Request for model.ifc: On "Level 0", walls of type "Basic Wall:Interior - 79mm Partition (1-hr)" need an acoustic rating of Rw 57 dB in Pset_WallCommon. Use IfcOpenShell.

First a look at what the model holds.

```python
import ifcopenshell
import ifcopenshell.util.element

model = ifcopenshell.open("model.ifc")
print(model.schema)
storey = next(s for s in model.by_type("IfcBuildingStorey") if s.Name == "Level 0")
walls = [e for e in ifcopenshell.util.element.get_decomposition(storey) if e.is_a("IfcWall")]
seen = {}
for e in walls:
    element_type = ifcopenshell.util.element.get_type(e)
    key = (element_type.Name if element_type != e and element_type else None, ifcopenshell.util.element.get_pset(e, "Pset_WallCommon", "AcousticRating"))
    seen[key] = seen.get(key, 0) + 1
for (name, value), count in sorted(seen.items(), key=str):
    print(count, "x", name, "|", value)
```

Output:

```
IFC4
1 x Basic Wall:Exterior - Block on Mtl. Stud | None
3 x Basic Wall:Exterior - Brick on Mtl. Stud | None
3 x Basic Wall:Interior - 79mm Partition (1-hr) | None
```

```python
import ifcopenshell
import ifcopenshell.api.pset
import ifcopenshell.util.element

model = ifcopenshell.open("model.ifc")

storey = next(s for s in model.by_type("IfcBuildingStorey") if s.Name == "Level 0")
walls = [e for e in ifcopenshell.util.element.get_decomposition(storey) if e.is_a("IfcWall")]

count = 0
for e in walls:
    element_type = ifcopenshell.util.element.get_type(e)
    if element_type in (None, e) or element_type.Name != "Basic Wall:Interior - 79mm Partition (1-hr)":
        continue
    # add_pset returns the element's existing set when there is one.
    pset = ifcopenshell.api.pset.add_pset(model, product=e, name="Pset_WallCommon")
    ifcopenshell.api.pset.edit_pset(model, pset=pset, properties={"AcousticRating": "Rw 57 dB"})
    count += 1

print(count, "walls updated")

model.write("model-out.ifc")
```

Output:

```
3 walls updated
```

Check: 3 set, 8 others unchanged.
